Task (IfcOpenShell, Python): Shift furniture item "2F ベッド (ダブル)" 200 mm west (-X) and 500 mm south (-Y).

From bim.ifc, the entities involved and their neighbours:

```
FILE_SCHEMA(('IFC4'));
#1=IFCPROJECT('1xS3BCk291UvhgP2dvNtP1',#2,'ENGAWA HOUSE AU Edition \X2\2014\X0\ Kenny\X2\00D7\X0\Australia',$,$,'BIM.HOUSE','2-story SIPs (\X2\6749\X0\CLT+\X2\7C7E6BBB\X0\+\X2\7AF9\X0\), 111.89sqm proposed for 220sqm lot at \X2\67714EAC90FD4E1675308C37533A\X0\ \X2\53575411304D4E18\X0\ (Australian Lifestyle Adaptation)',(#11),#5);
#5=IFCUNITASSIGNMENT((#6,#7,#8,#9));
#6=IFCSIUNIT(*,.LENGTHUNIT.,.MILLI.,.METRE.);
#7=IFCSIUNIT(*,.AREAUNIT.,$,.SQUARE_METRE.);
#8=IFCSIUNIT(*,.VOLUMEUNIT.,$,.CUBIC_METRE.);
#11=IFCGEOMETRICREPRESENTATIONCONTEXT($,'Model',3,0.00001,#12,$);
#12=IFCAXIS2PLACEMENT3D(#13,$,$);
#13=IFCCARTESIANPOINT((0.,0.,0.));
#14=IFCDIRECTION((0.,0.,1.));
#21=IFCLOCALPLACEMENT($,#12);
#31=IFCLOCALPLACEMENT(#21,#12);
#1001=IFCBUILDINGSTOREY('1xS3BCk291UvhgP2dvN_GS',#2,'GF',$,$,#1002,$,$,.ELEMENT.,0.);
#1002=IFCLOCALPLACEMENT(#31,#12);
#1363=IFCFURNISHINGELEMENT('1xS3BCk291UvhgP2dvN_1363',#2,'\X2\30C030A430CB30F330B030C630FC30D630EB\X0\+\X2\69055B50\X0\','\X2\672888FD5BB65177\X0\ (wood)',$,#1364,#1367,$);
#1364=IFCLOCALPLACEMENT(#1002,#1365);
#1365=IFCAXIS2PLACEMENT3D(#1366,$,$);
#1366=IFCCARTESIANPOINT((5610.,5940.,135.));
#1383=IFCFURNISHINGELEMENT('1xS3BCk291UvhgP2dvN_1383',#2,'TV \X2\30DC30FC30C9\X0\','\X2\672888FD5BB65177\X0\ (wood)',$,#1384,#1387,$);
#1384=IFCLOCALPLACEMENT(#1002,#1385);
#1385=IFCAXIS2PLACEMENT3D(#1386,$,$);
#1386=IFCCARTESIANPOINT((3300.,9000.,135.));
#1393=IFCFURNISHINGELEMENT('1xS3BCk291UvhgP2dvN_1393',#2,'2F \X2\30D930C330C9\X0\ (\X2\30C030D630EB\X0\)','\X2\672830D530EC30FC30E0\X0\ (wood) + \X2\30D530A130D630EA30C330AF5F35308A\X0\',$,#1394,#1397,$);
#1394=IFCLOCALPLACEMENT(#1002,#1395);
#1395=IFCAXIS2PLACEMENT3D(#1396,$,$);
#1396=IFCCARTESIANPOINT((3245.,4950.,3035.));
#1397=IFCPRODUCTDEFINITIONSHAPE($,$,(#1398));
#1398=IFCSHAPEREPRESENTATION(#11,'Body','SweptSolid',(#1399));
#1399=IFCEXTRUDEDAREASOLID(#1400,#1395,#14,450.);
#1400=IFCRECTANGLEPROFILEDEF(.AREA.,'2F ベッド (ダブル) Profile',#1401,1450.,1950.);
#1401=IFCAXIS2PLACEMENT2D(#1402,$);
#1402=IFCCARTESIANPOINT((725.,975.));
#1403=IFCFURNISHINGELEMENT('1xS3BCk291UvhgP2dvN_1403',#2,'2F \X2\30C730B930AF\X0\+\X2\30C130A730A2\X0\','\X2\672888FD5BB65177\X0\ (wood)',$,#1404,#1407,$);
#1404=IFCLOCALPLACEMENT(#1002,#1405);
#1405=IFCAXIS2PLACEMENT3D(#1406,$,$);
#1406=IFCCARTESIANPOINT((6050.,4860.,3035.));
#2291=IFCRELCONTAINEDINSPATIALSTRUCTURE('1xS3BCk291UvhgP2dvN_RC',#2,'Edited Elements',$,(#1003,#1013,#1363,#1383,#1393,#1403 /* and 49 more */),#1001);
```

```python
import ifcopenshell
import ifcopenshell.api.geometry
import ifcopenshell.util.placement

model = ifcopenshell.open("bim.ifc")

item = model.by_id(1393)
matrix = ifcopenshell.util.placement.get_local_placement(item.ObjectPlacement)
matrix[0, 3] -= 200.0
matrix[1, 3] -= 500.0
ifcopenshell.api.geometry.edit_object_placement(model, product=item, matrix=matrix, is_si=False)

print(ifcopenshell.util.placement.get_local_placement(item.ObjectPlacement).round(3) + 0.0)

model.write("bim_v2.ifc")
```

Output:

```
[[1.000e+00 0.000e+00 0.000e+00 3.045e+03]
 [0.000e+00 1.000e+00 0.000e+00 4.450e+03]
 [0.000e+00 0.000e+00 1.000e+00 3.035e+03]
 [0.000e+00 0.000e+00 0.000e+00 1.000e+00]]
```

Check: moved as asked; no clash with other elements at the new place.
